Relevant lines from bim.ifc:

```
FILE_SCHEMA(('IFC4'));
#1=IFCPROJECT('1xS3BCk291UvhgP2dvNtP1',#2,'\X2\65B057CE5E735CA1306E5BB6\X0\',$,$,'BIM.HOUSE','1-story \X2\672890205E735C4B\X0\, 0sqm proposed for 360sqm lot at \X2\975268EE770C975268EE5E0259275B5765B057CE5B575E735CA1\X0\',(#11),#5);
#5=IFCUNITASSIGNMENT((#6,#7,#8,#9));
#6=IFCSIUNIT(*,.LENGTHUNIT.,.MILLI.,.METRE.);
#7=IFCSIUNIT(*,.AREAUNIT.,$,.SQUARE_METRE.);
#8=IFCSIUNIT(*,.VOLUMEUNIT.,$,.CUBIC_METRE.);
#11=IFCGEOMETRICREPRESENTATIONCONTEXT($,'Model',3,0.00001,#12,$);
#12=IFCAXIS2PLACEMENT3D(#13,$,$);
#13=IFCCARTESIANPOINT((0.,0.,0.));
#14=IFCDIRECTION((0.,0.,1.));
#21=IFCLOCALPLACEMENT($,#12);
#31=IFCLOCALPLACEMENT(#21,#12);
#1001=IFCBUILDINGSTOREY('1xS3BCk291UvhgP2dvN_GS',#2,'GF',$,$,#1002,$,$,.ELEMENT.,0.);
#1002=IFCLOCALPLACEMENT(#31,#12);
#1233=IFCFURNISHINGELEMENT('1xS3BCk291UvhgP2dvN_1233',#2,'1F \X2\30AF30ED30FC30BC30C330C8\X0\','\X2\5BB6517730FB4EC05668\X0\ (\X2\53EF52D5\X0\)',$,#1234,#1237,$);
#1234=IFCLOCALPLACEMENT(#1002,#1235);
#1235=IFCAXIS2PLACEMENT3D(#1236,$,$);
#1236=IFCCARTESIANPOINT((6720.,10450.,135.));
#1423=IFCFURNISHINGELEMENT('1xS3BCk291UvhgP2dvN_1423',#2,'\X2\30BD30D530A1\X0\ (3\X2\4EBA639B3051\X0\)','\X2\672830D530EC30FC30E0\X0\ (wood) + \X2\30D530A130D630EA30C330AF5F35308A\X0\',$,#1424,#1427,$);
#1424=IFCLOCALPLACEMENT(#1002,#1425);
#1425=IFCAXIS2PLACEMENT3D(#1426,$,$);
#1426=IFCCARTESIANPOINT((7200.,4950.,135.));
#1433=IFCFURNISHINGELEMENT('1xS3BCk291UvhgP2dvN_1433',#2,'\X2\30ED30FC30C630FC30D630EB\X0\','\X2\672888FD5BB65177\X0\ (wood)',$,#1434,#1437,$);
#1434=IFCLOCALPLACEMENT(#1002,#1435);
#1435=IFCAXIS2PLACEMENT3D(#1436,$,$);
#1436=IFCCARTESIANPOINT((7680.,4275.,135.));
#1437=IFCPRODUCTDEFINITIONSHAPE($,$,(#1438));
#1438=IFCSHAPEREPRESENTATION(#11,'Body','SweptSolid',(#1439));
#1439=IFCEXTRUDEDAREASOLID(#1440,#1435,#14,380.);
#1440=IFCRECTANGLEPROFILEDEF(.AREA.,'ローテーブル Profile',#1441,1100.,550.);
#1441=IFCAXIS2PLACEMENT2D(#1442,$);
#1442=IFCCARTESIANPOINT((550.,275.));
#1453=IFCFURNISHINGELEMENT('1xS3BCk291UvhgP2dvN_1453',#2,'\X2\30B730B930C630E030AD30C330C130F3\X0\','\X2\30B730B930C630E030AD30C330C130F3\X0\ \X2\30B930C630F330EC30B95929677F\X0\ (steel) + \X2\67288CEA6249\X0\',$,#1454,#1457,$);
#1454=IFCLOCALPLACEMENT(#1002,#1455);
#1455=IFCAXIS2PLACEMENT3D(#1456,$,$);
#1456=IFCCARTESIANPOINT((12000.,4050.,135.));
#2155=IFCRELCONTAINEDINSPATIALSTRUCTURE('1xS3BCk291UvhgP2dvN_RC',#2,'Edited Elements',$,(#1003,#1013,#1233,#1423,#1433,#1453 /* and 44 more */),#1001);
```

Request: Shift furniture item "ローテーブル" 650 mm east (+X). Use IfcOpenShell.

```python
import ifcopenshell
import ifcopenshell.api.geometry
import ifcopenshell.util.placement
import ifcopenshell.util.unit

model = ifcopenshell.open("bim.ifc")
unit_scale = ifcopenshell.util.unit.calculate_unit_scale(model)

item = model.by_guid("1xS3BCk291UvhgP2dvN_1433")
matrix = ifcopenshell.util.placement.get_local_placement(item.ObjectPlacement)
matrix[0, 3] += 0.65 / unit_scale
ifcopenshell.api.geometry.edit_object_placement(model, product=item, matrix=matrix, is_si=False)

print(ifcopenshell.util.placement.get_local_placement(item.ObjectPlacement).round(3) + 0.0)

model.write("bim_v2.ifc")
```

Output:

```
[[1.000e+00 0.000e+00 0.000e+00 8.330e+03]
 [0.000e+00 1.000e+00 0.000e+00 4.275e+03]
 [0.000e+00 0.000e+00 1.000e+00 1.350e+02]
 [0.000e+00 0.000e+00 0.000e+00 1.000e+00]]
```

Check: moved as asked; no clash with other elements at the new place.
